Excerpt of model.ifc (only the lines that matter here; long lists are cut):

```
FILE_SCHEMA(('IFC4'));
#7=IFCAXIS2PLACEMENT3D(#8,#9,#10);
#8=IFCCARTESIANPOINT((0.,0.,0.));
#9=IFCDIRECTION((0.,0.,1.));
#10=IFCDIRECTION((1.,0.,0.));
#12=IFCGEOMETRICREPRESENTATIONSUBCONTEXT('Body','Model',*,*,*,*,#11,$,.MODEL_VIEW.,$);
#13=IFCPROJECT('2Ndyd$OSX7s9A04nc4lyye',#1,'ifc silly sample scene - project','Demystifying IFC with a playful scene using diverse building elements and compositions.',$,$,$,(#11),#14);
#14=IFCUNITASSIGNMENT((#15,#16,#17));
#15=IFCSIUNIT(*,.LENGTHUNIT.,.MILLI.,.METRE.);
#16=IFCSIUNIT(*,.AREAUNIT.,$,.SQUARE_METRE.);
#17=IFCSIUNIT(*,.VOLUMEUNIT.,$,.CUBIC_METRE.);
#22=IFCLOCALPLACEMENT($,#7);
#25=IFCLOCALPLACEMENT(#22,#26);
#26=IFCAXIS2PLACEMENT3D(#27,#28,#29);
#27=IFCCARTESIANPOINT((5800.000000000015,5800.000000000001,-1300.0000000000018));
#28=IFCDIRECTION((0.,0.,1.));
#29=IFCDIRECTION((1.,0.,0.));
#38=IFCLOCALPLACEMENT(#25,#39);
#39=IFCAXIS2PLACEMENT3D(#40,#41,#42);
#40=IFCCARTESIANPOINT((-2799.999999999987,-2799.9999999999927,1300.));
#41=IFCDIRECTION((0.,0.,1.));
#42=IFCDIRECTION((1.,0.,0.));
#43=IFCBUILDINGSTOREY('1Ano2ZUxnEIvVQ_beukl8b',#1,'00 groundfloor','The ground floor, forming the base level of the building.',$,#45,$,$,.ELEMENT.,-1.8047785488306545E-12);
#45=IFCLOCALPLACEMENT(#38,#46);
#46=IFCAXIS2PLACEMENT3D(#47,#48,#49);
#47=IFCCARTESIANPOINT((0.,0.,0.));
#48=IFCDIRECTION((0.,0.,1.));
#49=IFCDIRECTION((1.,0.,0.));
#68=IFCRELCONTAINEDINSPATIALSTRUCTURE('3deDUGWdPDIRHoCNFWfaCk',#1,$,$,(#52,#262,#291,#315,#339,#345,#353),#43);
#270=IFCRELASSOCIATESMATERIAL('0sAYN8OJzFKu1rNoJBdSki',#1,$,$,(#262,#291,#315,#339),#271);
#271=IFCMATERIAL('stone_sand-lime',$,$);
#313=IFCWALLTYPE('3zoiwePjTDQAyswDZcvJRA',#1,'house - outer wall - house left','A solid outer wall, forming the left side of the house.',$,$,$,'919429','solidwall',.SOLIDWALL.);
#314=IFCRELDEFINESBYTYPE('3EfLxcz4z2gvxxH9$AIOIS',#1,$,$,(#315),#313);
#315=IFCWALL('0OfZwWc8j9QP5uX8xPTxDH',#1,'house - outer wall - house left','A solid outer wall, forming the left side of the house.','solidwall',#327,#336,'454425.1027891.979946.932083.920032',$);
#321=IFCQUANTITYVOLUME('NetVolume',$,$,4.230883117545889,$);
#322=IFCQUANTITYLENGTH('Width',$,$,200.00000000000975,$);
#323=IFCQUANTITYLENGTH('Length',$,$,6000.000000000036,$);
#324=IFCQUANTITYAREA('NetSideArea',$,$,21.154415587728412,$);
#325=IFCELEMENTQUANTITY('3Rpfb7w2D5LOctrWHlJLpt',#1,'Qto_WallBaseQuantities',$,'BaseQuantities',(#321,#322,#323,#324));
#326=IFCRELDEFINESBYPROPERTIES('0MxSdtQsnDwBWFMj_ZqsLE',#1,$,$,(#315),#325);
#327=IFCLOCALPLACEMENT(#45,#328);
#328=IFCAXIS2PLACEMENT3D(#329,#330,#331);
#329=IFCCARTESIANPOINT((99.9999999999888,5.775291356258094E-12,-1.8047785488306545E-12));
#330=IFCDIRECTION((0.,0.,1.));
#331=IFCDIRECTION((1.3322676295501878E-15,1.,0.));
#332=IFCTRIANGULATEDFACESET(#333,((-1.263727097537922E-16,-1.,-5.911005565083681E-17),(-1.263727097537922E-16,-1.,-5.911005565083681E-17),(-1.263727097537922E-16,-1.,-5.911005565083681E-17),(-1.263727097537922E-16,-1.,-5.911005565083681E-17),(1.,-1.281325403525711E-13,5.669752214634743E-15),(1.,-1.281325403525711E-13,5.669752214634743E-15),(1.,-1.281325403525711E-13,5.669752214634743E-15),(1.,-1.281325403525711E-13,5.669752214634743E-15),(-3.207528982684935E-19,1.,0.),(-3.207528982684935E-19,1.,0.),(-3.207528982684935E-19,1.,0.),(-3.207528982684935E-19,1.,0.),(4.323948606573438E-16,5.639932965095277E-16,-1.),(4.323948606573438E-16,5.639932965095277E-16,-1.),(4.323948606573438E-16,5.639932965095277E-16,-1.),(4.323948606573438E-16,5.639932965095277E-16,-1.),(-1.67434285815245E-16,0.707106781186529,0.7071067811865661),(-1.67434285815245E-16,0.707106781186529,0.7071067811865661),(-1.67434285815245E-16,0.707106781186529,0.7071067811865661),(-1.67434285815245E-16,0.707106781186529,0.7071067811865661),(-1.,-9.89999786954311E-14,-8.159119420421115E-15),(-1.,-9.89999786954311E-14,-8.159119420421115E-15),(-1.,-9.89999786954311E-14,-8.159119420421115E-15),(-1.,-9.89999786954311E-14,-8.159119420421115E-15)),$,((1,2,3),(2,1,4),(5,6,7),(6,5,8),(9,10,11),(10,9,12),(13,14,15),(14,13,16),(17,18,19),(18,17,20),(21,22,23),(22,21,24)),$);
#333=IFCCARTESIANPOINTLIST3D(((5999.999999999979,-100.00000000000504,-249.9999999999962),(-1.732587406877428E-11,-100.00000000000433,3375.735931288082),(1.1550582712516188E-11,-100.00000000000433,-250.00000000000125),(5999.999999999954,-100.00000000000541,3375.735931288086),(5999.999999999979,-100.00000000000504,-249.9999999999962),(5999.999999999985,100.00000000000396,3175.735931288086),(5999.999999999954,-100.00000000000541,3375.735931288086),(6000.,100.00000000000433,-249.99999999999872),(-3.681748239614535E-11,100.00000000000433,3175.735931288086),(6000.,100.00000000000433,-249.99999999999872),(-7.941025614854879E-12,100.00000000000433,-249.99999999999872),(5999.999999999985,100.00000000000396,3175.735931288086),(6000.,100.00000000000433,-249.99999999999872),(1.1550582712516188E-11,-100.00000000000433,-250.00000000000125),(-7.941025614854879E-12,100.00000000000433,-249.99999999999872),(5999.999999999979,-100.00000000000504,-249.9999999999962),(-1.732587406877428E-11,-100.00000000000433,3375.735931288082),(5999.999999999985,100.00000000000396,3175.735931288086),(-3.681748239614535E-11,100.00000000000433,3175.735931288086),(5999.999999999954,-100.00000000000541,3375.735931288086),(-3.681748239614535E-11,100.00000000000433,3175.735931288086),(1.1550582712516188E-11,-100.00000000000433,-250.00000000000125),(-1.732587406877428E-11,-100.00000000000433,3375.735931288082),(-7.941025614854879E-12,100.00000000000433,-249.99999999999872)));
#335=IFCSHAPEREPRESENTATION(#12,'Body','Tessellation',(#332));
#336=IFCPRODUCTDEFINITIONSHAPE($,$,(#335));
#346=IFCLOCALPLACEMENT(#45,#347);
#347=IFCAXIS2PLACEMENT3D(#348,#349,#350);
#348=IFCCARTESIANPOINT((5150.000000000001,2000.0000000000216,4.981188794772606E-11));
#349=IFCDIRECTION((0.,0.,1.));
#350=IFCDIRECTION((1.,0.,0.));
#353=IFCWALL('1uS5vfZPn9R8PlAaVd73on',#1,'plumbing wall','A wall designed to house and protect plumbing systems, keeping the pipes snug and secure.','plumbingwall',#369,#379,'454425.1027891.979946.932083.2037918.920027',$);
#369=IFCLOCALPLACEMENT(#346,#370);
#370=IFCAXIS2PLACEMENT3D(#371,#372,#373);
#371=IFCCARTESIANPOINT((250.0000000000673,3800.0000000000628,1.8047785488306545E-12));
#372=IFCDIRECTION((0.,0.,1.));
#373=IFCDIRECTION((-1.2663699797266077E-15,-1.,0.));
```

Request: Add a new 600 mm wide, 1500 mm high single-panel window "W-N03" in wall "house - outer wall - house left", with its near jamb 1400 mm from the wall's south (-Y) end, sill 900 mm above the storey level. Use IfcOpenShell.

```python
import numpy as np
import ifcopenshell
import ifcopenshell.api.feature
import ifcopenshell.api.geometry
import ifcopenshell.api.pset
import ifcopenshell.api.root
import ifcopenshell.api.spatial
import ifcopenshell.geom
import ifcopenshell.util.element
import ifcopenshell.util.placement
import ifcopenshell.util.representation
import ifcopenshell.util.shape
import ifcopenshell.util.unit

model = ifcopenshell.open("model.ifc")
unit_scale = ifcopenshell.util.unit.calculate_unit_scale(model)
area_scale = ifcopenshell.util.unit.calculate_unit_scale(model, "AREAUNIT")
volume_scale = ifcopenshell.util.unit.calculate_unit_scale(model, "VOLUMEUNIT")
settings = ifcopenshell.geom.settings()


def volume(element):
    """Net volume in cubic metres, openings subtracted."""
    shape = ifcopenshell.geom.create_shape(settings, element)
    return ifcopenshell.util.shape.get_volume(shape.geometry)


wall = model.by_guid("0OfZwWc8j9QP5uX8xPTxDH")
storey = ifcopenshell.util.element.get_container(wall, ifc_class="IfcBuildingStorey")
context = ifcopenshell.util.representation.get_context(model, "Model", "Body", "MODEL_VIEW")
before = volume(wall)

width, height, from_end, sill = 0.6, 1.5, 1.4, 0.9  # metres

# The wall runs along its own X axis, and the end named is its -X end.
wall_shape = ifcopenshell.geom.create_shape(settings, wall)
x, y, z = ifcopenshell.util.shape.get_vertices(wall_shape.geometry).T
start = x.min() + from_end
face, thickness = float(y.min()), float(y.max() - y.min())
wall_matrix = ifcopenshell.util.placement.get_local_placement(wall.ObjectPlacement)
level = ifcopenshell.util.placement.get_local_placement(storey.ObjectPlacement)[2, 3]


def in_wall(x, y):
    """Placement at x, y metres in the wall's axes, at sill height."""
    matrix = wall_matrix.copy()
    matrix[:, 3] = wall_matrix @ np.array([x / unit_scale, y / unit_scale, 0.0, 1.0])
    matrix[2, 3] = level + sill / unit_scale
    return matrix


# Opening: a box that overshoots both wall faces by 50 mm.
opening = ifcopenshell.api.root.create_entity(model, ifc_class="IfcOpeningElement", predefined_type="OPENING")
box = ifcopenshell.api.geometry.add_wall_representation(
    model, context=context, length=width, height=height, thickness=thickness + 0.1
)
ifcopenshell.api.geometry.assign_representation(model, product=opening, representation=box)
ifcopenshell.api.geometry.edit_object_placement(model, product=opening, matrix=in_wall(start, face - 0.05), is_si=False)
ifcopenshell.api.feature.add_feature(model, feature=opening, element=wall)

window = ifcopenshell.api.root.create_entity(model, ifc_class="IfcWindow", name="W-N03", predefined_type="WINDOW")
window.OverallWidth, window.OverallHeight = width / unit_scale, height / unit_scale
window.PartitioningType = "SINGLE_PANEL"
body = ifcopenshell.api.geometry.add_window_representation(
    model,
    context=context,
    overall_width=window.OverallWidth,
    overall_height=window.OverallHeight,
    partition_type="SINGLE_PANEL",
)
ifcopenshell.api.geometry.assign_representation(model, product=window, representation=body)
ifcopenshell.api.spatial.assign_container(model, products=[window], relating_structure=storey)
ifcopenshell.api.feature.add_filling(model, opening=opening, element=window)

# Centre the window in the wall's thickness.
ifcopenshell.api.geometry.edit_object_placement(model, product=window, matrix=in_wall(start, face), is_si=False)
window_shape = ifcopenshell.geom.create_shape(settings, window)
depth = ifcopenshell.util.shape.get_vertices(window_shape.geometry)[:, 1]
offset = face + thickness / 2 - (depth.min() + depth.max()) / 2
ifcopenshell.api.geometry.edit_object_placement(model, product=window, matrix=in_wall(start, offset), is_si=False)

after = volume(wall)

# Update the wall's stored quantities.
qto = model.by_id(ifcopenshell.util.element.get_pset(wall, "Qto_WallBaseQuantities", should_inherit=False)["id"])
ifcopenshell.api.pset.edit_qto(model, qto=qto, properties={
    "NetVolume": after / volume_scale,
    "NetSideArea": after / thickness / area_scale,
})

print(f"wall volume {before:.3f} -> {after:.3f} m3")

model.write("model_edited.ifc")
```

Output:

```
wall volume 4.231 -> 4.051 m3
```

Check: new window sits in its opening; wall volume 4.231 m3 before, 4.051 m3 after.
